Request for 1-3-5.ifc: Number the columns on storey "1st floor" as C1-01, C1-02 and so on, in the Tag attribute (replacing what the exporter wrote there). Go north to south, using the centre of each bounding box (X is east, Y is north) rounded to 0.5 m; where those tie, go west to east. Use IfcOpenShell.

First a look at what the model holds.

```python
import ifcopenshell
import ifcopenshell.util.element
import ifcopenshell.util.placement

model = ifcopenshell.open("1-3-5.ifc")
print(model.schema)
storey = next(s for s in model.by_type("IfcBuildingStorey") if s.Name == "1st floor")
columns = [e for e in ifcopenshell.util.element.get_decomposition(storey) if e.is_a("IfcColumn")]
for e in sorted(columns, key=lambda e: e.id()):
    origin = ifcopenshell.util.placement.get_local_placement(e.ObjectPlacement)[:3, 3]
    print(e.id(), e.Tag, e.Name, origin.round(2) + 0.0, sep=" | ")
```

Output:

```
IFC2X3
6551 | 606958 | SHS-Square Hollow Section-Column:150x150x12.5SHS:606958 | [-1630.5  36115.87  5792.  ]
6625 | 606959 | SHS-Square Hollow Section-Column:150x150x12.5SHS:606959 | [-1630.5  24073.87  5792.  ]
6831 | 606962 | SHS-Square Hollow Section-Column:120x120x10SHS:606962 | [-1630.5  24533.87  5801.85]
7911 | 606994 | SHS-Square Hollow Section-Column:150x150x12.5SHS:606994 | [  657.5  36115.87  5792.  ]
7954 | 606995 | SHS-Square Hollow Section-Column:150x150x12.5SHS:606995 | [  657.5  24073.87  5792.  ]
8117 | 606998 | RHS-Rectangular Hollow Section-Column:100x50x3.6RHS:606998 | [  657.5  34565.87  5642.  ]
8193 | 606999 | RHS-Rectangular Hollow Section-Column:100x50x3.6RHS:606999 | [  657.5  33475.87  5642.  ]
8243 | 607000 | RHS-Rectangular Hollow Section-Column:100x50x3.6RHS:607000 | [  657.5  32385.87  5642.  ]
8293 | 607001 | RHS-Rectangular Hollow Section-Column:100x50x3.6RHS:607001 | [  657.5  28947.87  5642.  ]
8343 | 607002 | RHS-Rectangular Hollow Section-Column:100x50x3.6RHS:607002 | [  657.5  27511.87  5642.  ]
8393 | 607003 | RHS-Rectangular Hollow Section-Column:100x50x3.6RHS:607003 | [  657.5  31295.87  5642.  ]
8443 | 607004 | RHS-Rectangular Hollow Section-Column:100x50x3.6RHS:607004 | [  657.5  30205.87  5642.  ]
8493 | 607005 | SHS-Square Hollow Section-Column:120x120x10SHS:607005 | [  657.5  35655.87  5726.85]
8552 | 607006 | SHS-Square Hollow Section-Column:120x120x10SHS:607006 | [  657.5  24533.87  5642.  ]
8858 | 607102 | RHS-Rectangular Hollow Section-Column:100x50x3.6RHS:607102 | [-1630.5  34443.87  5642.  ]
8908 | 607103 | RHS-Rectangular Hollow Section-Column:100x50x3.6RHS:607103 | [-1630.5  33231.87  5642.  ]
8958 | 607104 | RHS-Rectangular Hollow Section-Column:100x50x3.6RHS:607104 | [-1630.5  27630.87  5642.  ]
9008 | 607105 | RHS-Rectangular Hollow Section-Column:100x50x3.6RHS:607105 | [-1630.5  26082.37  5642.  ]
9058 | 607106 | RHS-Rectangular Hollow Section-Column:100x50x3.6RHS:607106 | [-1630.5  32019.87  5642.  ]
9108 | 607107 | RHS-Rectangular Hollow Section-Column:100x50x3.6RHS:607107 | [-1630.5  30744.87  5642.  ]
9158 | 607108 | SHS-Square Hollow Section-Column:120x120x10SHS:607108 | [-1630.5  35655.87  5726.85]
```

```python
import ifcopenshell
import ifcopenshell.geom
import ifcopenshell.util.element
import ifcopenshell.util.shape

model = ifcopenshell.open("1-3-5.ifc")
settings = ifcopenshell.geom.settings()
settings.set("use-world-coords", True)


def centre(element):
    shape = ifcopenshell.geom.create_shape(settings, element)
    return ifcopenshell.util.shape.get_bbox_centroid(shape.geometry)


storey = next(s for s in model.by_type("IfcBuildingStorey") if s.Name == "1st floor")
columns = [e for e in ifcopenshell.util.element.get_decomposition(storey) if e.is_a("IfcColumn")]

# Insertion points can sit at a corner or the storey origin, so sort by the geometry (in metres).
centres = {e: centre(e) for e in columns}
columns.sort(key=lambda e: (-round(centres[e][1] / 0.5), centres[e][0]))

for i, e in enumerate(columns, start=1):
    number = f"C1-{i:02d}"
    e.Tag = number
    print(e.id(), number)

model.write("1-3-5_rev.ifc")
```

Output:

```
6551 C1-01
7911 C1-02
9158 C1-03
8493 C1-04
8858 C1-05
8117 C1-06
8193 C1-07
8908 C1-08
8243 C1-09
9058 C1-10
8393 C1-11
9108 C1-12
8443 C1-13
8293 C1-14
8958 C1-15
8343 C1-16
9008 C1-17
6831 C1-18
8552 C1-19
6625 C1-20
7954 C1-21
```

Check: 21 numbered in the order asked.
